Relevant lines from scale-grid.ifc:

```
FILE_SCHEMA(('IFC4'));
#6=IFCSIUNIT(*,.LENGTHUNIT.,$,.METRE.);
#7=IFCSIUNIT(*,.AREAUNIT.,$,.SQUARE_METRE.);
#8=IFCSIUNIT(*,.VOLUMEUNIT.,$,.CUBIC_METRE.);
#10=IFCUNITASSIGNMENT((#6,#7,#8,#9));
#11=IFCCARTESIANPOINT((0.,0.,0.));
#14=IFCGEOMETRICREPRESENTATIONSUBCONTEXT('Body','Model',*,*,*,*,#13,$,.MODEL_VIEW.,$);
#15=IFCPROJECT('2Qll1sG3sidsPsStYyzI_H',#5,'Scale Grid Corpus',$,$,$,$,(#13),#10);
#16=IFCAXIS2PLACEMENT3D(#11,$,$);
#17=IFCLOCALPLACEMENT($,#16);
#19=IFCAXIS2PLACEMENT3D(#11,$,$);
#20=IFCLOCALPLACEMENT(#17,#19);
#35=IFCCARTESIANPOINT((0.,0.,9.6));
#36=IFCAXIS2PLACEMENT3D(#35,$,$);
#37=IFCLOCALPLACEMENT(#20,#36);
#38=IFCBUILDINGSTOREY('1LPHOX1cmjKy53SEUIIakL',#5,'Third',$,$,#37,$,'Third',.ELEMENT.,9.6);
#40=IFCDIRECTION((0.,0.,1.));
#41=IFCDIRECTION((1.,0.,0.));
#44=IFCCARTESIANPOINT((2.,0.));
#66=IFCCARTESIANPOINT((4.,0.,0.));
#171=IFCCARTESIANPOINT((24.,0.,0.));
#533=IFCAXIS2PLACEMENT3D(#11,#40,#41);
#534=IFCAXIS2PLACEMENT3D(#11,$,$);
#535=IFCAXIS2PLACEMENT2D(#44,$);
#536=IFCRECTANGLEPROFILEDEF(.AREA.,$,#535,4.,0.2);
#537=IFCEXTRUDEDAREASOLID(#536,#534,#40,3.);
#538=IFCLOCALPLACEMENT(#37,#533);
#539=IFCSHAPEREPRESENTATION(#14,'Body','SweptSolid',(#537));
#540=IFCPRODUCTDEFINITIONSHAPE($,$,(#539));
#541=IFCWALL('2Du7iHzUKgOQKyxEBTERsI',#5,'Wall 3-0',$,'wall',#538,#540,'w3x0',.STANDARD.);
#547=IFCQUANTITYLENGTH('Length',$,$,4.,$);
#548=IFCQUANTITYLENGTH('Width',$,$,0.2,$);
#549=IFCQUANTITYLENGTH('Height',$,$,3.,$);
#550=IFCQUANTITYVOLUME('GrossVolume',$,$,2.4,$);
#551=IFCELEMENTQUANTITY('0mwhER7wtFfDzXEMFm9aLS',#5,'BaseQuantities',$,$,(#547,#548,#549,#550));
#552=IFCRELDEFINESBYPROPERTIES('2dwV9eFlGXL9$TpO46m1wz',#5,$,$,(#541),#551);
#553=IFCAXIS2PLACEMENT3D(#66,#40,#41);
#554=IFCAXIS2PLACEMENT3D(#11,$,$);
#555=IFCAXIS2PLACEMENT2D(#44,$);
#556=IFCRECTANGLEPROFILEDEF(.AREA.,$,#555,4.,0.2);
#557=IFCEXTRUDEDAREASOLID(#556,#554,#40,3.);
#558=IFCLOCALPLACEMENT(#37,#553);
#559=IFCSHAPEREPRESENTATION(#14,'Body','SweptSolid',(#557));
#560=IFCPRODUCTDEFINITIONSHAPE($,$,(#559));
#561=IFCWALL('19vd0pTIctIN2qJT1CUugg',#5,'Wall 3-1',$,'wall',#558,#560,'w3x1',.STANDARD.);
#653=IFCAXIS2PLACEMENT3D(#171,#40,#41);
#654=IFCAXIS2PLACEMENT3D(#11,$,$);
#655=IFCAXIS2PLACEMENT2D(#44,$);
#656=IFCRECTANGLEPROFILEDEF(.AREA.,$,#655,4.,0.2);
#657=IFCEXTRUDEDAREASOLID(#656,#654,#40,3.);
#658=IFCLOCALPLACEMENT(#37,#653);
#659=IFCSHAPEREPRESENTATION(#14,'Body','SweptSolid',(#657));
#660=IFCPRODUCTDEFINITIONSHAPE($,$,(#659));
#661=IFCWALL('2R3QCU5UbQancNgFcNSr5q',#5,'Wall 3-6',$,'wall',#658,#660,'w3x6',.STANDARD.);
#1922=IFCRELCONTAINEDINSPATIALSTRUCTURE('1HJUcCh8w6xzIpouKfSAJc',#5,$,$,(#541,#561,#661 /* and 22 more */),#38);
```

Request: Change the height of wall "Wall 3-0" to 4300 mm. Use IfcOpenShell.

```python
import ifcopenshell
import ifcopenshell.api.pset
import ifcopenshell.geom
import ifcopenshell.util.element
import ifcopenshell.util.representation
import ifcopenshell.util.shape
import ifcopenshell.util.unit

model = ifcopenshell.open("scale-grid.ifc")
unit_scale = ifcopenshell.util.unit.calculate_unit_scale(model)
volume_scale = ifcopenshell.util.unit.calculate_unit_scale(model, "VOLUMEUNIT")
settings = ifcopenshell.geom.settings()


def volume(element):
    """Net volume in cubic metres, openings subtracted."""
    shape = ifcopenshell.geom.create_shape(settings, element)
    return ifcopenshell.util.shape.get_volume(shape.geometry)


wall = model.by_guid("2Du7iHzUKgOQKyxEBTERsI")
before = volume(wall)

body = ifcopenshell.util.representation.get_representation(wall, "Model", "Body")
solid = body.Items[0]
old_height = solid.Depth
solid.Depth = 4.3 / unit_scale
after = volume(wall)

# Update the stored height, areas and volumes.
qto = model.by_id(ifcopenshell.util.element.get_pset(wall, "BaseQuantities", should_inherit=False)["id"])
ifcopenshell.api.pset.edit_qto(model, qto=qto, properties={
    "Height": solid.Depth,
    "GrossVolume": ifcopenshell.util.element.get_pset(wall, "BaseQuantities", "GrossVolume") * solid.Depth / old_height,
})

print(f"height {old_height:g} -> {solid.Depth:g}, volume {before:.3f} -> {after:.3f} m3")

model.write("scale-grid-out.ifc")
```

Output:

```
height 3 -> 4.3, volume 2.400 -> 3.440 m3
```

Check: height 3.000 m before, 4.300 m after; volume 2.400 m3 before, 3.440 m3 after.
